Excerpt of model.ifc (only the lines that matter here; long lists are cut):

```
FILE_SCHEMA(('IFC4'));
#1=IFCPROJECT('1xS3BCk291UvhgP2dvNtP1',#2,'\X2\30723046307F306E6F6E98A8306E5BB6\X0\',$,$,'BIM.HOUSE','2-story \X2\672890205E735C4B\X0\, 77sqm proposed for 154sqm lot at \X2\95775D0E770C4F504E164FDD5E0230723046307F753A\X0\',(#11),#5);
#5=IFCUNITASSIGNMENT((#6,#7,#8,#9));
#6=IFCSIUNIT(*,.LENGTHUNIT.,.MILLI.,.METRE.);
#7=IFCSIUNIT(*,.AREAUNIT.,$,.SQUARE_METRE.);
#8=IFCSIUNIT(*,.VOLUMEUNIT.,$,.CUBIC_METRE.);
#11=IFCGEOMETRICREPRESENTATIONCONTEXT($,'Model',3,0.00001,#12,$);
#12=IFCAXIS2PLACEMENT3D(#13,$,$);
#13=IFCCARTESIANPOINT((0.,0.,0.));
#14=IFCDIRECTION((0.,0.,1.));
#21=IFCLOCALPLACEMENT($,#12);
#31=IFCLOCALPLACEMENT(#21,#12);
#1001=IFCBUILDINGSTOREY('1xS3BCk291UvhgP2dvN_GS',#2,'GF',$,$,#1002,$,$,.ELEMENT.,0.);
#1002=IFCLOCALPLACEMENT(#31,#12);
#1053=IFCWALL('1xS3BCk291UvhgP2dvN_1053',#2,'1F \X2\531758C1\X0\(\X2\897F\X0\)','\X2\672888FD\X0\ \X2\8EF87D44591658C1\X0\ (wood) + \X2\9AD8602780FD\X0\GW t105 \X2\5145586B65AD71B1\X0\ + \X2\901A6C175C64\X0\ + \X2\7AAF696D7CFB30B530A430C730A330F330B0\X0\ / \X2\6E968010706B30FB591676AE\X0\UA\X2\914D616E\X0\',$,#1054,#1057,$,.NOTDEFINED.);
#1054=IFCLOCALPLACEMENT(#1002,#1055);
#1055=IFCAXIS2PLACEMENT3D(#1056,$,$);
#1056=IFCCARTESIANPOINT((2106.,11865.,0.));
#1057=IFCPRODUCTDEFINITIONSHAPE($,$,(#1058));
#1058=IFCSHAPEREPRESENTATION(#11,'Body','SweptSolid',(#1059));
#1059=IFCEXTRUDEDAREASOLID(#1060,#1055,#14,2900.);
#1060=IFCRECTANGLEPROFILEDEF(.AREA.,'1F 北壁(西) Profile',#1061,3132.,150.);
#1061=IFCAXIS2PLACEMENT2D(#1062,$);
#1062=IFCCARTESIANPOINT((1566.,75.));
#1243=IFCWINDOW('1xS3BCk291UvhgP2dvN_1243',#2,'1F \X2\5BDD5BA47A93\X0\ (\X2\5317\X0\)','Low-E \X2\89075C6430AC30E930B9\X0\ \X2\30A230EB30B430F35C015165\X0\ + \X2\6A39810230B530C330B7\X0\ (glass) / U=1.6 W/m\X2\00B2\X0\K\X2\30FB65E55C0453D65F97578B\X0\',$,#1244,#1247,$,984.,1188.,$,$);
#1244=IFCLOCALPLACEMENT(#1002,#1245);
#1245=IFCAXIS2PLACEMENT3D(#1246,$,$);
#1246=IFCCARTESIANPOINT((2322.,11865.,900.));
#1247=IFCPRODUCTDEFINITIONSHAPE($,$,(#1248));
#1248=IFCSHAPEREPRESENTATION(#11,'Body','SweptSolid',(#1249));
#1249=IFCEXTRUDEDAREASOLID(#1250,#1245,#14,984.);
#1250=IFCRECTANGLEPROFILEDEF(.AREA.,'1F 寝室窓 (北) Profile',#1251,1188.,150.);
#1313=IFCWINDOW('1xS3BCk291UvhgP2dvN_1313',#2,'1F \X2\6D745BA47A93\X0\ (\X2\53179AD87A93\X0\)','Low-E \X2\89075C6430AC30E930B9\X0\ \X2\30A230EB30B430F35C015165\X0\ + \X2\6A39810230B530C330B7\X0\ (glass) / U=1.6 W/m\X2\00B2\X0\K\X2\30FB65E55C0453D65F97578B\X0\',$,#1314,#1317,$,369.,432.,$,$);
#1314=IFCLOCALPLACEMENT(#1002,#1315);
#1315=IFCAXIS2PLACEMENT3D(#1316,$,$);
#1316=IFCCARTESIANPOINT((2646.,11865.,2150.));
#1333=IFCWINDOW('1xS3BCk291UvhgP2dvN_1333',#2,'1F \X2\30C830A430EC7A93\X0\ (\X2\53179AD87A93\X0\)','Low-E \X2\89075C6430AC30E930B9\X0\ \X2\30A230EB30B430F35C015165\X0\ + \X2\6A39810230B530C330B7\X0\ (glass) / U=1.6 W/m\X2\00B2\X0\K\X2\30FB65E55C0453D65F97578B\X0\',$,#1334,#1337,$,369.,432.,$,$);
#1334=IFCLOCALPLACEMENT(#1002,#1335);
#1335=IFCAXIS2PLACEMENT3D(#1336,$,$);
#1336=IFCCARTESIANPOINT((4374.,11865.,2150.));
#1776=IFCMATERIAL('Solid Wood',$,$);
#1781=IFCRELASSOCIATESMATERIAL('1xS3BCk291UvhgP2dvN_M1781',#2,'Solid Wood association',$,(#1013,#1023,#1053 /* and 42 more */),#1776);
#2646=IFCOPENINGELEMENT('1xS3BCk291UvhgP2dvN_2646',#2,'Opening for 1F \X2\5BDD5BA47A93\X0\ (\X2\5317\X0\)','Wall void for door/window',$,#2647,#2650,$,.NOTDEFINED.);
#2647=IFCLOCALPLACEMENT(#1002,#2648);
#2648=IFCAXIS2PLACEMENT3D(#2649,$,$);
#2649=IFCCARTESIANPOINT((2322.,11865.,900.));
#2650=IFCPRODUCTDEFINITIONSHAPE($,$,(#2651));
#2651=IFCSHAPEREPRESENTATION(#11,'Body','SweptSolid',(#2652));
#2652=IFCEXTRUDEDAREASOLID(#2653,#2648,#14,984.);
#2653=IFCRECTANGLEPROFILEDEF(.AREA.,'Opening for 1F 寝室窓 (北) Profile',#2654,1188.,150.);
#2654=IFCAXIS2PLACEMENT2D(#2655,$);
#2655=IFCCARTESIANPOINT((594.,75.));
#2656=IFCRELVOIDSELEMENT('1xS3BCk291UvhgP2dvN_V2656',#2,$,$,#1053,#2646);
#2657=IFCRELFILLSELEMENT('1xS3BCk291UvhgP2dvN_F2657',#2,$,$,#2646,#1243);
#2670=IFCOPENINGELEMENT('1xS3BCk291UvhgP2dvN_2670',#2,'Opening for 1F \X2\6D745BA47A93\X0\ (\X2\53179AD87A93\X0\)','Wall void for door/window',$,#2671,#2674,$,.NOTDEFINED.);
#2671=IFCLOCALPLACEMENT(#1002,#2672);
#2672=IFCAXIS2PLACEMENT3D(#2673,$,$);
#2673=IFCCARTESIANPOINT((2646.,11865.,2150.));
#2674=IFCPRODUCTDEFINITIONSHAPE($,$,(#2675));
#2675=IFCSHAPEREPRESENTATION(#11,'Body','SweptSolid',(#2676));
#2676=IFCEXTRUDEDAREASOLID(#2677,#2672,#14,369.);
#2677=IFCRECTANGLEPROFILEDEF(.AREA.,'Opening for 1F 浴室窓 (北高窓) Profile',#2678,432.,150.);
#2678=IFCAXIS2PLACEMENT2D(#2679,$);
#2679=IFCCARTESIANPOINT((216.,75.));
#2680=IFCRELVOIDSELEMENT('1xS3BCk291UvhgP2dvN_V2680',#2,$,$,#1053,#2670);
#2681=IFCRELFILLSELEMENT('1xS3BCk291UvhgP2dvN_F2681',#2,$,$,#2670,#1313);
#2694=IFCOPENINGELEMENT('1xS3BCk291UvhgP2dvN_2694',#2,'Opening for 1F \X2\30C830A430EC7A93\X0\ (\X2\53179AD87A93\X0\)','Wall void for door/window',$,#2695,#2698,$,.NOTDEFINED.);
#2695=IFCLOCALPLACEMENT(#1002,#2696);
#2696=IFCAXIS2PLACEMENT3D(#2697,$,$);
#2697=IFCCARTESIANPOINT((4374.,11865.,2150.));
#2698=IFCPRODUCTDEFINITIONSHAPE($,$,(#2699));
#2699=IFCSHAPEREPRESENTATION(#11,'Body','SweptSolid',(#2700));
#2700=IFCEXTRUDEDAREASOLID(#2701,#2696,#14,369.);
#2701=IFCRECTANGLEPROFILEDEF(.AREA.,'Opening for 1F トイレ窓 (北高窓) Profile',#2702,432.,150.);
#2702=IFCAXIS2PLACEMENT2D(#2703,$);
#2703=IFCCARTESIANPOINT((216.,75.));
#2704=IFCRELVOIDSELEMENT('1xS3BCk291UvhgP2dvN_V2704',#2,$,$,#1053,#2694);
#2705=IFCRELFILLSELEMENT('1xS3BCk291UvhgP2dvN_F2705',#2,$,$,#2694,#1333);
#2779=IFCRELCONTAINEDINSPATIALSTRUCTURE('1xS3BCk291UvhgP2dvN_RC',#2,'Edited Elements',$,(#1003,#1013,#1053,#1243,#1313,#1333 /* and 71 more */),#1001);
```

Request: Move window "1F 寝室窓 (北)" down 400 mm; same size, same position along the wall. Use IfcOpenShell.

```python
import numpy as np
import ifcopenshell
import ifcopenshell.api.geometry
import ifcopenshell.util.placement
import ifcopenshell.util.unit

model = ifcopenshell.open("model.ifc")
unit_scale = ifcopenshell.util.unit.calculate_unit_scale(model)

window = model.by_guid("1xS3BCk291UvhgP2dvN_1243")
opening = window.FillsVoids[0].RelatingOpeningElement
dz = -400.0

shift = np.array([0.0, 0.0, dz])
# The window is not placed relative to its opening, so move both.
for product in (opening, window):
    matrix = ifcopenshell.util.placement.get_local_placement(product.ObjectPlacement)
    matrix[:3, 3] += shift
    ifcopenshell.api.geometry.edit_object_placement(model, product=product, matrix=matrix, is_si=False)

print(f"moved by {dz * unit_scale:+.3f} m")

model.write("model_edited.ifc")
```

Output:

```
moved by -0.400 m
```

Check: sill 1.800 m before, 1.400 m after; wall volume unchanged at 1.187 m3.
